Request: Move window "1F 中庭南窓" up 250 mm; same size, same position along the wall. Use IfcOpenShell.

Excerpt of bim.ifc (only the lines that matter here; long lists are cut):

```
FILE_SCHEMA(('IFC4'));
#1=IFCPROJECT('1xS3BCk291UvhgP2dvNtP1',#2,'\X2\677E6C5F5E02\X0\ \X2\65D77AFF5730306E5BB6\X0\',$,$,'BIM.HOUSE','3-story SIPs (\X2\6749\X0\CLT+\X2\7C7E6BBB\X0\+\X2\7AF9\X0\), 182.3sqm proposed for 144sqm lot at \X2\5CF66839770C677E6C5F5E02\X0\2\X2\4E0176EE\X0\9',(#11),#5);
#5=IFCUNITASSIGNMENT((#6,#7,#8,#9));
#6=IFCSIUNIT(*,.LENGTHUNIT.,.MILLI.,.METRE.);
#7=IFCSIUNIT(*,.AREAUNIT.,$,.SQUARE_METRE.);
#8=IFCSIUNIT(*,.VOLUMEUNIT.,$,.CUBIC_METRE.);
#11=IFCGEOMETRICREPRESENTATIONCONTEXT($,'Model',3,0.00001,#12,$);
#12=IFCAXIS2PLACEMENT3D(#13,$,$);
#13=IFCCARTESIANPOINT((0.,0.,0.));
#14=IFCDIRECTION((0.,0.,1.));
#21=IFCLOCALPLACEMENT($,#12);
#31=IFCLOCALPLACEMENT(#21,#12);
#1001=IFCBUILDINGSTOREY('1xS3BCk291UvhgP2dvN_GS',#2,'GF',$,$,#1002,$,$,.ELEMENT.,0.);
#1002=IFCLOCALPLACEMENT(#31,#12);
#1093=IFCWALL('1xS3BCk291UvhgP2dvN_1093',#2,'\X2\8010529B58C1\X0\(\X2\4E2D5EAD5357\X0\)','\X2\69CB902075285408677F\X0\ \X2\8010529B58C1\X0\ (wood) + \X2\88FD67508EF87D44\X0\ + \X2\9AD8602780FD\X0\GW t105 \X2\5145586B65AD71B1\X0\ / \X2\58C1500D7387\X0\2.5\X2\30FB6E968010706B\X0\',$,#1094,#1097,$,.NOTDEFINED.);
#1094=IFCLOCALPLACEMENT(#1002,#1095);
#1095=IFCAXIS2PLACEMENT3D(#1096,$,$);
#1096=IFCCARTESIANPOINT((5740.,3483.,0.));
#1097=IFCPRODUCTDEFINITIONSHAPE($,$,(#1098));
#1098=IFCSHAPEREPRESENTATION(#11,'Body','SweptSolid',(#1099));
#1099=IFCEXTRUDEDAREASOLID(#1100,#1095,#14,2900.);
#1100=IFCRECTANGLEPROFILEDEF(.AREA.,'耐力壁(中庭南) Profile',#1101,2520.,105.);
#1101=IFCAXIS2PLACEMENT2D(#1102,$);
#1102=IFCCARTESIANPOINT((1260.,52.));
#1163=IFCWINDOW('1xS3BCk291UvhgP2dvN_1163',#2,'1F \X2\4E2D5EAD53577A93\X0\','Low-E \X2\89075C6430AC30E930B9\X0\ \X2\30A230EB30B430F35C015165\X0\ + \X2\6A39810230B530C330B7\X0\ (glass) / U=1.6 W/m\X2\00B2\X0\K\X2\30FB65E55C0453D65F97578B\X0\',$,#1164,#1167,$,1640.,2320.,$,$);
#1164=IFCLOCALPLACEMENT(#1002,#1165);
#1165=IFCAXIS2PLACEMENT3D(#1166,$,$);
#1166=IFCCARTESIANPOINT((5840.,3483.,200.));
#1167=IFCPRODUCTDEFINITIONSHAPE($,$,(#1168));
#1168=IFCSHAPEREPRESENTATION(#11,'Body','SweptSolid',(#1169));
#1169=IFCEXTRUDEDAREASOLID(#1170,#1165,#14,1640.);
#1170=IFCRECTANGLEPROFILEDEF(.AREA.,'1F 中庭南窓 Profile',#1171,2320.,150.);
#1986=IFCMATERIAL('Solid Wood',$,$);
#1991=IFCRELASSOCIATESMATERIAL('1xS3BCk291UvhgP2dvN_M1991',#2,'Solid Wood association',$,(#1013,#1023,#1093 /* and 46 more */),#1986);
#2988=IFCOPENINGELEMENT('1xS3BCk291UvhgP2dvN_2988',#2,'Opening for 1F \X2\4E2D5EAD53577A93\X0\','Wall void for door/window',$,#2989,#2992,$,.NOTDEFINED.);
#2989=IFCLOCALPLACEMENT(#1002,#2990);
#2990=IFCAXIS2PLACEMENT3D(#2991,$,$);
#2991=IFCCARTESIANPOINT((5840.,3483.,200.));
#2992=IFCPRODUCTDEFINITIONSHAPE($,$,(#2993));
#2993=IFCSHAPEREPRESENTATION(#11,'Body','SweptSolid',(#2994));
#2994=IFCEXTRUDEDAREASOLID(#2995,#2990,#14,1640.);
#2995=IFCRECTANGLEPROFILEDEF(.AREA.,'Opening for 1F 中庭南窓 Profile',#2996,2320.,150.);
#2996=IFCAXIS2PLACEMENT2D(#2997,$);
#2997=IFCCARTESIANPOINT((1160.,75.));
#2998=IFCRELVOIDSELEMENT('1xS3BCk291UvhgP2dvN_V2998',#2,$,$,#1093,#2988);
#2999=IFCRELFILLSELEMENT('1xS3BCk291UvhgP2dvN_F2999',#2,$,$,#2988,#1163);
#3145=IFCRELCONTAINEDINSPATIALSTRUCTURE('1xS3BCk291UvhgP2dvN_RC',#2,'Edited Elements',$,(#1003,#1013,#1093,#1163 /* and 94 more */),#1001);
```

```python
import numpy as np
import ifcopenshell
import ifcopenshell.api.geometry
import ifcopenshell.util.placement
import ifcopenshell.util.unit

model = ifcopenshell.open("bim.ifc")
unit_scale = ifcopenshell.util.unit.calculate_unit_scale(model)

window = model.by_id(1163)
opening = window.FillsVoids[0].RelatingOpeningElement
dz = 0.25 / unit_scale

shift = np.array([0.0, 0.0, dz])
# The window is not placed relative to its opening, so move both.
for product in (opening, window):
    matrix = ifcopenshell.util.placement.get_local_placement(product.ObjectPlacement)
    matrix[:3, 3] += shift
    ifcopenshell.api.geometry.edit_object_placement(model, product=product, matrix=matrix, is_si=False)

print(f"moved by {dz * unit_scale:+.3f} m")

model.write("bim_edited.ifc")
```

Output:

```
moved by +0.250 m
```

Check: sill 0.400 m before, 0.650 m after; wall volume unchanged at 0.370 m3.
